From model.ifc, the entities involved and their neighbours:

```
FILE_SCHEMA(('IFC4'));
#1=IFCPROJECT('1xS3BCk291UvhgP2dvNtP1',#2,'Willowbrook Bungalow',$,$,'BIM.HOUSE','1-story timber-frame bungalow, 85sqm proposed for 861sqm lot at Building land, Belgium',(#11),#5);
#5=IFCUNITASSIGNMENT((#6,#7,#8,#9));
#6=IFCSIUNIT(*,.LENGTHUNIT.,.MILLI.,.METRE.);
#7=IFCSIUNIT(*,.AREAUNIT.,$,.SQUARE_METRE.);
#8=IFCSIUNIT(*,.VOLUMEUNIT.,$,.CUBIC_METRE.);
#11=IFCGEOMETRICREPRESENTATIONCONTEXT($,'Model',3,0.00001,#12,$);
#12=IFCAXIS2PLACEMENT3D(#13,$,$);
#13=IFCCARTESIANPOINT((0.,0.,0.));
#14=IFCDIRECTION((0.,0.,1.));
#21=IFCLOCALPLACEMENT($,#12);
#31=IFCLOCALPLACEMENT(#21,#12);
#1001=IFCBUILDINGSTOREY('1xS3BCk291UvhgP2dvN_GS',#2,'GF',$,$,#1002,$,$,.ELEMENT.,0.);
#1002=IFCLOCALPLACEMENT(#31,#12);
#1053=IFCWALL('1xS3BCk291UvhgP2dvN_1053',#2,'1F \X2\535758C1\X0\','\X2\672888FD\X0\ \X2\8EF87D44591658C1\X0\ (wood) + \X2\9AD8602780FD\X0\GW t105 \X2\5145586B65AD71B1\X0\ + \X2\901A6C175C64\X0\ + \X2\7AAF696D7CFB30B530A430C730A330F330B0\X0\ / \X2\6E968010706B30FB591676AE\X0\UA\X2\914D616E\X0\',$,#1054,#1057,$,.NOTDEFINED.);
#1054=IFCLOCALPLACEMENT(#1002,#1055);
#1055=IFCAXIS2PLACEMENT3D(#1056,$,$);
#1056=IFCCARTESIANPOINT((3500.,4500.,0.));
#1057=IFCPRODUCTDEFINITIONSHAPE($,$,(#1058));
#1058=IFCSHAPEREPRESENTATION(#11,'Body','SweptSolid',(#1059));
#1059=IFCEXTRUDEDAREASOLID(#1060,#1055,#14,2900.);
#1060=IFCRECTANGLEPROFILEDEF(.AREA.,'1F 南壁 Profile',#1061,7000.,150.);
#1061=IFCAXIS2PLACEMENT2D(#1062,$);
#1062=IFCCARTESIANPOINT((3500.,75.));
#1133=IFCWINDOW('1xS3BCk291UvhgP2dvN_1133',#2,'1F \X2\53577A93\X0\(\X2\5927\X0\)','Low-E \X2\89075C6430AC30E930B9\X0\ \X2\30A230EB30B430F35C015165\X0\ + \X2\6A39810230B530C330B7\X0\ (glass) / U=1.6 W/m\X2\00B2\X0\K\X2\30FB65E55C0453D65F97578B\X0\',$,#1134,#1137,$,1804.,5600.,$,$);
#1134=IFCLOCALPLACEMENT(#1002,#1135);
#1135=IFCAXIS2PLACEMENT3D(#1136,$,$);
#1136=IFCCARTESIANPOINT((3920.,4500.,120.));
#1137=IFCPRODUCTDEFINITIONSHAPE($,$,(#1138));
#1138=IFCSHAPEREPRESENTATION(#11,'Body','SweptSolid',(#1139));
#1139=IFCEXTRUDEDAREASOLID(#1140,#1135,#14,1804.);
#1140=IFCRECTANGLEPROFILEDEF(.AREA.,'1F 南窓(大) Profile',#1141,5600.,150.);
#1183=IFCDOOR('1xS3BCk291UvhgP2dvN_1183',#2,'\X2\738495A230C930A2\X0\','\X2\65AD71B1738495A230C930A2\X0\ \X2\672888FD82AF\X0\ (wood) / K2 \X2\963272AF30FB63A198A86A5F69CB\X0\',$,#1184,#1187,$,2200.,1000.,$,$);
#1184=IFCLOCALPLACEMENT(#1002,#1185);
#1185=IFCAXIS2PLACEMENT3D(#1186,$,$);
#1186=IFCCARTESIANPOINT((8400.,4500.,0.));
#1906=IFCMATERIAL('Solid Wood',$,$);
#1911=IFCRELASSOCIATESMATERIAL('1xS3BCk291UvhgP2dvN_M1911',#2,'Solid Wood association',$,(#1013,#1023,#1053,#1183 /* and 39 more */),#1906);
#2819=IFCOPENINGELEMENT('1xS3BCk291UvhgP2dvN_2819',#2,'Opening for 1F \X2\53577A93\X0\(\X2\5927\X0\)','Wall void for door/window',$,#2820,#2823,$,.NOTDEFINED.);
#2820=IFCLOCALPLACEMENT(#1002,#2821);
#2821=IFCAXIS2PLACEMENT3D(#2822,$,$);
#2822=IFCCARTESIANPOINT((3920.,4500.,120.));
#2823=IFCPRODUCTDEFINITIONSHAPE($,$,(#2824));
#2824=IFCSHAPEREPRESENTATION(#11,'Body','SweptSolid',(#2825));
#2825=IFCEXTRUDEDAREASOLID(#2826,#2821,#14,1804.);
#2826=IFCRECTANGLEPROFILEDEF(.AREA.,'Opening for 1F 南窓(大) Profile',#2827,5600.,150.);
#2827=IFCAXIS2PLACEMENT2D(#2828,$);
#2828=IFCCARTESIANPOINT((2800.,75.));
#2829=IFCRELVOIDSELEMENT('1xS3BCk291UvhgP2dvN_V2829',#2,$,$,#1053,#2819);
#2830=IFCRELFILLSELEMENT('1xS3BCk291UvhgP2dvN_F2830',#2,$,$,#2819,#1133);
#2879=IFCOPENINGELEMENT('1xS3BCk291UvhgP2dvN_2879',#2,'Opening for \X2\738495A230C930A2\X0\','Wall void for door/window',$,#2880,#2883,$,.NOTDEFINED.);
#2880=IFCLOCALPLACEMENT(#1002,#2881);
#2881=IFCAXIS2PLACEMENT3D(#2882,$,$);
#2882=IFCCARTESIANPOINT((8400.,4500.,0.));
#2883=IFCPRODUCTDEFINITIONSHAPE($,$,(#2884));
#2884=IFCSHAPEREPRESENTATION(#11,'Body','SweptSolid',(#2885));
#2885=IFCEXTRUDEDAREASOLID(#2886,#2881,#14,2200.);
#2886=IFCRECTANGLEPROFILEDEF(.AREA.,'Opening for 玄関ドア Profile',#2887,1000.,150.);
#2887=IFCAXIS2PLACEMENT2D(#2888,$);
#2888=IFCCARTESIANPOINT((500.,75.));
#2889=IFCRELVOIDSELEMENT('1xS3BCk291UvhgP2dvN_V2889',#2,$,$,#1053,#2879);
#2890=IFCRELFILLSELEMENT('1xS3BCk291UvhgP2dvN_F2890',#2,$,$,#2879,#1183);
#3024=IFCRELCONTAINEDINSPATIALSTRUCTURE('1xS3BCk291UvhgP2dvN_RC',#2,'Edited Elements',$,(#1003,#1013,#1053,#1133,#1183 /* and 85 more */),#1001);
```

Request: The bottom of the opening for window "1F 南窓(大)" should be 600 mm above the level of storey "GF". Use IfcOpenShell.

```python
import numpy as np
import ifcopenshell
import ifcopenshell.api.geometry
import ifcopenshell.geom
import ifcopenshell.util.element
import ifcopenshell.util.placement
import ifcopenshell.util.shape
import ifcopenshell.util.unit

model = ifcopenshell.open("model.ifc")
unit_scale = ifcopenshell.util.unit.calculate_unit_scale(model)

window = model.by_guid("1xS3BCk291UvhgP2dvN_1133")
opening = window.FillsVoids[0].RelatingOpeningElement
storey = ifcopenshell.util.element.get_container(window, ifc_class="IfcBuildingStorey")
level = ifcopenshell.util.placement.get_local_placement(storey.ObjectPlacement)[2, 3]

# The opening's origin need not be at the sill, so measure its lowest point.
shape = ifcopenshell.geom.create_shape(ifcopenshell.geom.settings(), opening)
bottom = ifcopenshell.util.shape.get_shape_bottom_elevation(shape, shape.geometry) / unit_scale
dz = level + 600.0 - bottom

shift = np.array([0.0, 0.0, dz])
# The window is not placed relative to its opening, so move both.
for product in (opening, window):
    matrix = ifcopenshell.util.placement.get_local_placement(product.ObjectPlacement)
    matrix[:3, 3] += shift
    ifcopenshell.api.geometry.edit_object_placement(model, product=product, matrix=matrix, is_si=False)

print(f"moved by {dz * unit_scale:+.3f} m")

model.write("model_updated.ifc")
```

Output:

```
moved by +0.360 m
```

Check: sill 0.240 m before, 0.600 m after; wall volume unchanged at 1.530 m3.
